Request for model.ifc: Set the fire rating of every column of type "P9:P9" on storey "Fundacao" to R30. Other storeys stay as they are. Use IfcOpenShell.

First a look at what the model holds.

```python
import ifcopenshell
import ifcopenshell.util.element

model = ifcopenshell.open("model.ifc")
print(model.schema)
storey = next(s for s in model.by_type("IfcBuildingStorey") if s.Name == "Fundacao")
columns = [e for e in ifcopenshell.util.element.get_decomposition(storey) if e.is_a("IfcColumn")]
seen = {}
for e in columns:
    element_type = ifcopenshell.util.element.get_type(e)
    key = (element_type.Name if element_type != e and element_type else None, ifcopenshell.util.element.get_pset(e, "Pset_ColumnCommon", "FireRating"))
    seen[key] = seen.get(key, 0) + 1
for (name, value), count in sorted(seen.items(), key=str):
    print(count, "x", name, "|", value)
```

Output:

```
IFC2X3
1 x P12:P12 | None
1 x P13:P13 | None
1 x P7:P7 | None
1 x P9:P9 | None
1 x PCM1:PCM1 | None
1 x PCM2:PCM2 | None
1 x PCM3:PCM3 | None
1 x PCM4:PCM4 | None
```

```python
import ifcopenshell
import ifcopenshell.api.pset
import ifcopenshell.util.element

model = ifcopenshell.open("model.ifc")

storey = next(s for s in model.by_type("IfcBuildingStorey") if s.Name == "Fundacao")
columns = [e for e in ifcopenshell.util.element.get_decomposition(storey) if e.is_a("IfcColumn")]

count = 0
for e in columns:
    element_type = ifcopenshell.util.element.get_type(e)
    if element_type in (None, e) or element_type.Name != "P9:P9":
        continue
    # add_pset returns the element's existing set when there is one.
    pset = ifcopenshell.api.pset.add_pset(model, product=e, name="Pset_ColumnCommon")
    ifcopenshell.api.pset.edit_pset(model, pset=pset, properties={"FireRating": "R30"})
    count += 1

print(count, "columns updated")

model.write("model_v2.ifc")
```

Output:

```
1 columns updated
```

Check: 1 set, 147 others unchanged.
